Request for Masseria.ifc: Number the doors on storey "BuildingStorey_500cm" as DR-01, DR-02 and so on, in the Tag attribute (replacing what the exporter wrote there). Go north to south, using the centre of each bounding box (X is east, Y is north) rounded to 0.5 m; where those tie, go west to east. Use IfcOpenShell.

First a look at what the model holds.

```python
import ifcopenshell
import ifcopenshell.util.element
import ifcopenshell.util.placement

model = ifcopenshell.open("Masseria.ifc")
print(model.schema)
storey = next(s for s in model.by_type("IfcBuildingStorey") if s.Name == "BuildingStorey_500cm")
doors = [e for e in ifcopenshell.util.element.get_decomposition(storey) if e.is_a("IfcDoor")]
for e in sorted(doors, key=lambda e: e.id()):
    origin = ifcopenshell.util.placement.get_local_placement(e.ObjectPlacement)[:3, 3]
    print(e.id(), e.Tag, e.Name, origin.round(2) + 0.0, sep=" | ")
```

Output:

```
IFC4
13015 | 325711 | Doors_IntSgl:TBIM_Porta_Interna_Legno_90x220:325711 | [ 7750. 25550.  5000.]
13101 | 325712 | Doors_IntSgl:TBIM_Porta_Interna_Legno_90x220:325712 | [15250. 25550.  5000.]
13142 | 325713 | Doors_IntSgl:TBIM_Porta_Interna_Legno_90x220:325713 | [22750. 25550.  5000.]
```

```python
import ifcopenshell
import ifcopenshell.geom
import ifcopenshell.util.element
import ifcopenshell.util.shape

model = ifcopenshell.open("Masseria.ifc")
settings = ifcopenshell.geom.settings()
settings.set("use-world-coords", True)


def centre(element):
    shape = ifcopenshell.geom.create_shape(settings, element)
    return ifcopenshell.util.shape.get_bbox_centroid(shape.geometry)


storey = next(s for s in model.by_type("IfcBuildingStorey") if s.Name == "BuildingStorey_500cm")
doors = [e for e in ifcopenshell.util.element.get_decomposition(storey) if e.is_a("IfcDoor")]

# Insertion points can sit at a corner or the storey origin, so sort by the geometry (in metres).
centres = {e: centre(e) for e in doors}
doors.sort(key=lambda e: (-round(centres[e][1] / 0.5), centres[e][0]))

for i, e in enumerate(doors, start=1):
    number = f"DR-{i:02d}"
    e.Tag = number
    print(e.id(), number)

model.write("Masseria_v2.ifc")
```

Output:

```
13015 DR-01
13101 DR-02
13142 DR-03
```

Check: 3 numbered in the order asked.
